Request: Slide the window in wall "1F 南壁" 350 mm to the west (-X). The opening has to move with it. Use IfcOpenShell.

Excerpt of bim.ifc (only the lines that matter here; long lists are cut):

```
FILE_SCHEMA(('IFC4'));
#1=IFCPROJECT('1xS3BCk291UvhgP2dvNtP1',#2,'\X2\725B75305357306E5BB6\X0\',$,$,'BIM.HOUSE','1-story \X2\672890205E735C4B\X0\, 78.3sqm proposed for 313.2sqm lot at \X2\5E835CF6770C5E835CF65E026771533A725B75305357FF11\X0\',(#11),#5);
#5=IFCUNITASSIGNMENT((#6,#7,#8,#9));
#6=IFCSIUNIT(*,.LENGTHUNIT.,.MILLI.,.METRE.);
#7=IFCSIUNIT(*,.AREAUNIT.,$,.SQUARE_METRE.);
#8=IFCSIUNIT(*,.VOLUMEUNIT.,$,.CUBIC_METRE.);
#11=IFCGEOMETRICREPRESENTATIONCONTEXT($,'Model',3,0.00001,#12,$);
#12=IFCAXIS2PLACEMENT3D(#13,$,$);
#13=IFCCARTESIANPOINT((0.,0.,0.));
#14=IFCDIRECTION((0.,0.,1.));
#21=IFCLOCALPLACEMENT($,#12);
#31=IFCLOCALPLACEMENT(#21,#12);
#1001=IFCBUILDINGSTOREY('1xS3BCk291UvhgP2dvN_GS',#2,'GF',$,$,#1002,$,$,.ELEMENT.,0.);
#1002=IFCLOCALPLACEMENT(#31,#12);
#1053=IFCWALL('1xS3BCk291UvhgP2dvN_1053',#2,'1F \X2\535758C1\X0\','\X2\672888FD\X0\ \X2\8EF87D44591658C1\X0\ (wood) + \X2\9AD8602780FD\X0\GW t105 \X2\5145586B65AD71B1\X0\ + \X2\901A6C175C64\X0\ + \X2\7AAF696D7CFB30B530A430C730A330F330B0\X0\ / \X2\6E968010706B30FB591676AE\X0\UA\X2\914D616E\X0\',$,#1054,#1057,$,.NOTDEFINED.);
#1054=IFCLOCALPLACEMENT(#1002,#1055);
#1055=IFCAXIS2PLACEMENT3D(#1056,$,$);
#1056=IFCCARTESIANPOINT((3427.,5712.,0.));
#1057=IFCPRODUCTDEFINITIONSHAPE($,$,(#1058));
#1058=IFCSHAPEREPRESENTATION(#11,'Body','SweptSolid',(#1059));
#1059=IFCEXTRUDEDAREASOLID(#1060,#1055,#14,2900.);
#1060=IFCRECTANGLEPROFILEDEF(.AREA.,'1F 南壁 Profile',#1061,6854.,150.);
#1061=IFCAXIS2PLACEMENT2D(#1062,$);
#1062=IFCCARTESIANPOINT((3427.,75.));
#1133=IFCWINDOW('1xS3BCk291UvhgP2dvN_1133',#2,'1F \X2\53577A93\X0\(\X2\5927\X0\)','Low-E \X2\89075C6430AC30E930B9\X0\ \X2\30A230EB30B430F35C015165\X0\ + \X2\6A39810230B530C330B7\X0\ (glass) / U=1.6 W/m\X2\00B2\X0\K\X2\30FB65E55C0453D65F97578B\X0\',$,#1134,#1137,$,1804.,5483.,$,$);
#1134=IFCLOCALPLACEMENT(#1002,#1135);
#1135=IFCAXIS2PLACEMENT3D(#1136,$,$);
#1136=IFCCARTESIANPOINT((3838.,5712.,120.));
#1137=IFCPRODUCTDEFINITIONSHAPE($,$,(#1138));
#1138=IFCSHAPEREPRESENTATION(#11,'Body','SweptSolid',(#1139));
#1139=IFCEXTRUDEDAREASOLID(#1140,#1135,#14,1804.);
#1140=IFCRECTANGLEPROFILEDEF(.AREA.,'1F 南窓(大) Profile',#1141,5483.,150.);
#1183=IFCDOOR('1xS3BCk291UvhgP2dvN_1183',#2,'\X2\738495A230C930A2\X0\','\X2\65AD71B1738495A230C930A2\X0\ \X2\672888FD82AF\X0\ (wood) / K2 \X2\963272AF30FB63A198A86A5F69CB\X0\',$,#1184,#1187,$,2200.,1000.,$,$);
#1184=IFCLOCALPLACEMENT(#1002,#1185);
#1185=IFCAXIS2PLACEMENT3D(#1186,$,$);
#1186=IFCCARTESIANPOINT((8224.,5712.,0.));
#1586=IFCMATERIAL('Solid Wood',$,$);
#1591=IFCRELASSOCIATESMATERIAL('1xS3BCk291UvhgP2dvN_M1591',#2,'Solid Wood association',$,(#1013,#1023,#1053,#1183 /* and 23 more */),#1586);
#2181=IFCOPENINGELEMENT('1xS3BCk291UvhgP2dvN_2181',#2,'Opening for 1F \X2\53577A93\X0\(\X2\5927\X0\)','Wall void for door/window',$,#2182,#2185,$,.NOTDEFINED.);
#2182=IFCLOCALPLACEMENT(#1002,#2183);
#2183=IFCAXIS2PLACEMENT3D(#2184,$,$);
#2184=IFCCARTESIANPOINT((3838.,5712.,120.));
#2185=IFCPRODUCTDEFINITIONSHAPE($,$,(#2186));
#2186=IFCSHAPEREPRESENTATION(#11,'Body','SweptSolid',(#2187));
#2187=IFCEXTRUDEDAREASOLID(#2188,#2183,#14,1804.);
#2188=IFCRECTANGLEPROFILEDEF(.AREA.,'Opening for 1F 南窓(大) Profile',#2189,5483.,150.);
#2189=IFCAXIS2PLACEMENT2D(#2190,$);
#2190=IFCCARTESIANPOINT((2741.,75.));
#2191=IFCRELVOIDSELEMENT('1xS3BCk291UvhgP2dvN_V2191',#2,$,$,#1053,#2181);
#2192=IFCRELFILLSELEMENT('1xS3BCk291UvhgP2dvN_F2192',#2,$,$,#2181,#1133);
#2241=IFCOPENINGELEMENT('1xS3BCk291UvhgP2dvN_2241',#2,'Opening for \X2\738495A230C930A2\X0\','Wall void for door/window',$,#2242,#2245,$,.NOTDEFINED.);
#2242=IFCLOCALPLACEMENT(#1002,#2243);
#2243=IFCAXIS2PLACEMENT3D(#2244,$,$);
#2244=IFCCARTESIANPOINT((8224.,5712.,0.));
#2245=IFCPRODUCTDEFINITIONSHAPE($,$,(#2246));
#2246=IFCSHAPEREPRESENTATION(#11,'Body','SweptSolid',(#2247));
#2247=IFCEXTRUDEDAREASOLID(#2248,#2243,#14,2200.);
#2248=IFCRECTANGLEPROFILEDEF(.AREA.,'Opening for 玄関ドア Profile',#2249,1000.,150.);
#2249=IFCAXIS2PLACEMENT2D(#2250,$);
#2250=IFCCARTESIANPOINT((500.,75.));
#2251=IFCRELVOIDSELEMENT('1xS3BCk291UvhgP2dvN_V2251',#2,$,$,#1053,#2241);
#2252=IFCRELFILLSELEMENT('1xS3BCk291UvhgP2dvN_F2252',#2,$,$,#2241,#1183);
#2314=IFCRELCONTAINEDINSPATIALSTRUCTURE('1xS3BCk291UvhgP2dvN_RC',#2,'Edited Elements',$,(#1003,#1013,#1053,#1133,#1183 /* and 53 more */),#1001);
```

```python
import ifcopenshell
import ifcopenshell.api.geometry
import ifcopenshell.util.placement

model = ifcopenshell.open("bim.ifc")

window = model.by_guid("1xS3BCk291UvhgP2dvN_1133")
opening = window.FillsVoids[0].RelatingOpeningElement
wall = opening.VoidsElements[0].RelatingBuildingElement

wall_matrix = ifcopenshell.util.placement.get_local_placement(wall.ObjectPlacement)
shift = wall_matrix[:3, 0] * -350.0
before = ifcopenshell.util.placement.get_local_placement(window.ObjectPlacement)[:3, 3].copy()

# The window is not placed relative to its opening, so move both.
for product in (opening, window):
    matrix = ifcopenshell.util.placement.get_local_placement(product.ObjectPlacement)
    matrix[:3, 3] += shift
    ifcopenshell.api.geometry.edit_object_placement(model, product=product, matrix=matrix, is_si=False)

after = ifcopenshell.util.placement.get_local_placement(window.ObjectPlacement)[:3, 3]
print("window moved by", (after - before).round(3) + 0.0)

model.write("bim_updated.ifc")
```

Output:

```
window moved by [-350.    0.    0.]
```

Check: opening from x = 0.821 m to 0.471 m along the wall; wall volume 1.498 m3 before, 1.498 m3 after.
